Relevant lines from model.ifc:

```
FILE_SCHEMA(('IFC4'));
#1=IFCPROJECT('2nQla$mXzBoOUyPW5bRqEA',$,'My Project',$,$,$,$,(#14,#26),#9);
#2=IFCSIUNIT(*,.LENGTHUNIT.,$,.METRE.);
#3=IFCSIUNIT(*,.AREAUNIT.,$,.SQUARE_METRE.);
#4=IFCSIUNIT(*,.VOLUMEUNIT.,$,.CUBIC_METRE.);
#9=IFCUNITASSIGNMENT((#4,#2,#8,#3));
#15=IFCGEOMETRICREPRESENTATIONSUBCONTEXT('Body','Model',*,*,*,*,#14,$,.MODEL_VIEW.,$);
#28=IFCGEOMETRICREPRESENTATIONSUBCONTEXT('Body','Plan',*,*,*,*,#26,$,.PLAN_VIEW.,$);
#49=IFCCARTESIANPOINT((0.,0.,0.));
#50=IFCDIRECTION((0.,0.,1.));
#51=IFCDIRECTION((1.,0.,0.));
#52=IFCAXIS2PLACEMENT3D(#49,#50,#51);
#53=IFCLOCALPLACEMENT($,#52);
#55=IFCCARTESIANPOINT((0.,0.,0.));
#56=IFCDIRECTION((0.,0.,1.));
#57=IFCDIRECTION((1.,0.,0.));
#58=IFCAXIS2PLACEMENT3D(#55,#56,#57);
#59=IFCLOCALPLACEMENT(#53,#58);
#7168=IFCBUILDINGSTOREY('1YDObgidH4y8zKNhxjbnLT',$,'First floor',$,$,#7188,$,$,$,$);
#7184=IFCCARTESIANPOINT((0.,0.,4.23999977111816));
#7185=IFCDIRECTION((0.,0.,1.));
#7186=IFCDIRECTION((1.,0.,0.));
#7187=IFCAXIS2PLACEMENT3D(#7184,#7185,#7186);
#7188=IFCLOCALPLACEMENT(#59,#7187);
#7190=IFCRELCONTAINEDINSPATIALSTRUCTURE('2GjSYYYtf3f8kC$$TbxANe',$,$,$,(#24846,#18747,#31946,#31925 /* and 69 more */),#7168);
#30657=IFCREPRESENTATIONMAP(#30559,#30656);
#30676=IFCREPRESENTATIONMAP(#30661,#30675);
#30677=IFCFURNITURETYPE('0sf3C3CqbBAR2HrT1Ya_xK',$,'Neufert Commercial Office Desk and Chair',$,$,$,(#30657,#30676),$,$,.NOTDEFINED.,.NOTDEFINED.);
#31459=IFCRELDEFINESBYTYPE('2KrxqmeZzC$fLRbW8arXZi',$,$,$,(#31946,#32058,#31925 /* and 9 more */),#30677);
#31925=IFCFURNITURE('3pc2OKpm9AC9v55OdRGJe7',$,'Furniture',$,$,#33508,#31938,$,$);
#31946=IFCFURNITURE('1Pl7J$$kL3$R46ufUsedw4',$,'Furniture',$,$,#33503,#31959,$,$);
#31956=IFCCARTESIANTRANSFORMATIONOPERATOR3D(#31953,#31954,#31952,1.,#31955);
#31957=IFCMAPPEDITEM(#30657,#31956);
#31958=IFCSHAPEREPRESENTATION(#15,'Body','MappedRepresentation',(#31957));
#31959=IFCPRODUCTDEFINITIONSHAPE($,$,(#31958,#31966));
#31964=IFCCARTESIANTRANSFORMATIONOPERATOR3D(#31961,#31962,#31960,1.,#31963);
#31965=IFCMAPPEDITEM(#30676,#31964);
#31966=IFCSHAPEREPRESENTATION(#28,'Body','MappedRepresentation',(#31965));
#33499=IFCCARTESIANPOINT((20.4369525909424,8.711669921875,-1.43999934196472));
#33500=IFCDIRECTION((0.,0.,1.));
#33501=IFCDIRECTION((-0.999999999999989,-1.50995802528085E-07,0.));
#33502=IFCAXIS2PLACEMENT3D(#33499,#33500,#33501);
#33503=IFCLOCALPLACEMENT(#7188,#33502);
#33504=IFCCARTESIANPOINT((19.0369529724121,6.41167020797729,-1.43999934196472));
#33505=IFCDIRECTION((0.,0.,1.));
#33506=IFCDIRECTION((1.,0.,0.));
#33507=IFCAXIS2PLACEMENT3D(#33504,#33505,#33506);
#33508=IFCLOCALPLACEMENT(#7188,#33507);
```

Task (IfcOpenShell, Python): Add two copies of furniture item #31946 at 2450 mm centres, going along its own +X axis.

```python
import ifcopenshell
import ifcopenshell.api.geometry
import ifcopenshell.api.root
import ifcopenshell.util.element
import ifcopenshell.util.placement
import ifcopenshell.util.unit

model = ifcopenshell.open("model.ifc")
unit_scale = ifcopenshell.util.unit.calculate_unit_scale(model)

source = model.by_guid("1Pl7J$$kL3$R46ufUsedw4")
base = ifcopenshell.util.placement.get_local_placement(source.ObjectPlacement)
step = base[:3, 0] * 2.45 / unit_scale

for i in range(1, 3):
    copy = ifcopenshell.api.root.copy_class(model, product=source)
    copy.Representation = ifcopenshell.util.element.copy_deep(
        model, source.Representation, exclude=["IfcGeometricRepresentationContext", "IfcRepresentationMap"]
    )
    matrix = base.copy()
    matrix[:3, 3] += i * step
    print("added at", matrix[:3, 3].round(3) + 0.0)
    ifcopenshell.api.geometry.edit_object_placement(model, product=copy, matrix=matrix, is_si=False)

model.write("model_rev.ifc")
```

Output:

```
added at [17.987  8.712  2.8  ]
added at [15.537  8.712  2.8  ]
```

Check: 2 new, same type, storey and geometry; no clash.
